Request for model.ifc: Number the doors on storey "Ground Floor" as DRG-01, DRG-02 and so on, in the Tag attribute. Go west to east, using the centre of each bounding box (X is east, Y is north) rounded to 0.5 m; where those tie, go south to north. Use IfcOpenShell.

First a look at what the model holds.

```python
import ifcopenshell
import ifcopenshell.util.element
import ifcopenshell.util.placement

model = ifcopenshell.open("model.ifc")
print(model.schema)
storey = next(s for s in model.by_type("IfcBuildingStorey") if s.Name == "Ground Floor")
doors = [e for e in ifcopenshell.util.element.get_decomposition(storey) if e.is_a("IfcDoor")]
for e in sorted(doors, key=lambda e: e.id()):
    origin = ifcopenshell.util.placement.get_local_placement(e.ObjectPlacement)[:3, 3]
    print(e.id(), e.Tag, e.Name, origin.round(2) + 0.0, sep=" | ")
```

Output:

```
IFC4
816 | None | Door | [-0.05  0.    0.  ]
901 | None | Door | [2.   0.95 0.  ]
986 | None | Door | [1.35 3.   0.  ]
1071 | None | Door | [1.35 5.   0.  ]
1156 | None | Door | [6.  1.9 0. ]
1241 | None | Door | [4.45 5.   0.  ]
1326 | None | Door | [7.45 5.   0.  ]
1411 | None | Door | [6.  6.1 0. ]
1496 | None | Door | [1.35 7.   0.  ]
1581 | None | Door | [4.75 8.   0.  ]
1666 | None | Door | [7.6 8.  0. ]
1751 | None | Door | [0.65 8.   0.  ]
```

```python
import ifcopenshell
import ifcopenshell.geom
import ifcopenshell.util.element
import ifcopenshell.util.shape

model = ifcopenshell.open("model.ifc")
settings = ifcopenshell.geom.settings()
settings.set("use-world-coords", True)


def centre(element):
    shape = ifcopenshell.geom.create_shape(settings, element)
    return ifcopenshell.util.shape.get_bbox_centroid(shape.geometry)


storey = next(s for s in model.by_type("IfcBuildingStorey") if s.Name == "Ground Floor")
doors = [e for e in ifcopenshell.util.element.get_decomposition(storey) if e.is_a("IfcDoor")]

# Insertion points can sit at a corner or the storey origin, so sort by the geometry (in metres).
centres = {e: centre(e) for e in doors}
doors.sort(key=lambda e: (round(centres[e][0] / 0.5), centres[e][1]))

for i, e in enumerate(doors, start=1):
    number = f"DRG-{i:02d}"
    e.Tag = number
    print(e.id(), number)

model.write("model-out.ifc")
```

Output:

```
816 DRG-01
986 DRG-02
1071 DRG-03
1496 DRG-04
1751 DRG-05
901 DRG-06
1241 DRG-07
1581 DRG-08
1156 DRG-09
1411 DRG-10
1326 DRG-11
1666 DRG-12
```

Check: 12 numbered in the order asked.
